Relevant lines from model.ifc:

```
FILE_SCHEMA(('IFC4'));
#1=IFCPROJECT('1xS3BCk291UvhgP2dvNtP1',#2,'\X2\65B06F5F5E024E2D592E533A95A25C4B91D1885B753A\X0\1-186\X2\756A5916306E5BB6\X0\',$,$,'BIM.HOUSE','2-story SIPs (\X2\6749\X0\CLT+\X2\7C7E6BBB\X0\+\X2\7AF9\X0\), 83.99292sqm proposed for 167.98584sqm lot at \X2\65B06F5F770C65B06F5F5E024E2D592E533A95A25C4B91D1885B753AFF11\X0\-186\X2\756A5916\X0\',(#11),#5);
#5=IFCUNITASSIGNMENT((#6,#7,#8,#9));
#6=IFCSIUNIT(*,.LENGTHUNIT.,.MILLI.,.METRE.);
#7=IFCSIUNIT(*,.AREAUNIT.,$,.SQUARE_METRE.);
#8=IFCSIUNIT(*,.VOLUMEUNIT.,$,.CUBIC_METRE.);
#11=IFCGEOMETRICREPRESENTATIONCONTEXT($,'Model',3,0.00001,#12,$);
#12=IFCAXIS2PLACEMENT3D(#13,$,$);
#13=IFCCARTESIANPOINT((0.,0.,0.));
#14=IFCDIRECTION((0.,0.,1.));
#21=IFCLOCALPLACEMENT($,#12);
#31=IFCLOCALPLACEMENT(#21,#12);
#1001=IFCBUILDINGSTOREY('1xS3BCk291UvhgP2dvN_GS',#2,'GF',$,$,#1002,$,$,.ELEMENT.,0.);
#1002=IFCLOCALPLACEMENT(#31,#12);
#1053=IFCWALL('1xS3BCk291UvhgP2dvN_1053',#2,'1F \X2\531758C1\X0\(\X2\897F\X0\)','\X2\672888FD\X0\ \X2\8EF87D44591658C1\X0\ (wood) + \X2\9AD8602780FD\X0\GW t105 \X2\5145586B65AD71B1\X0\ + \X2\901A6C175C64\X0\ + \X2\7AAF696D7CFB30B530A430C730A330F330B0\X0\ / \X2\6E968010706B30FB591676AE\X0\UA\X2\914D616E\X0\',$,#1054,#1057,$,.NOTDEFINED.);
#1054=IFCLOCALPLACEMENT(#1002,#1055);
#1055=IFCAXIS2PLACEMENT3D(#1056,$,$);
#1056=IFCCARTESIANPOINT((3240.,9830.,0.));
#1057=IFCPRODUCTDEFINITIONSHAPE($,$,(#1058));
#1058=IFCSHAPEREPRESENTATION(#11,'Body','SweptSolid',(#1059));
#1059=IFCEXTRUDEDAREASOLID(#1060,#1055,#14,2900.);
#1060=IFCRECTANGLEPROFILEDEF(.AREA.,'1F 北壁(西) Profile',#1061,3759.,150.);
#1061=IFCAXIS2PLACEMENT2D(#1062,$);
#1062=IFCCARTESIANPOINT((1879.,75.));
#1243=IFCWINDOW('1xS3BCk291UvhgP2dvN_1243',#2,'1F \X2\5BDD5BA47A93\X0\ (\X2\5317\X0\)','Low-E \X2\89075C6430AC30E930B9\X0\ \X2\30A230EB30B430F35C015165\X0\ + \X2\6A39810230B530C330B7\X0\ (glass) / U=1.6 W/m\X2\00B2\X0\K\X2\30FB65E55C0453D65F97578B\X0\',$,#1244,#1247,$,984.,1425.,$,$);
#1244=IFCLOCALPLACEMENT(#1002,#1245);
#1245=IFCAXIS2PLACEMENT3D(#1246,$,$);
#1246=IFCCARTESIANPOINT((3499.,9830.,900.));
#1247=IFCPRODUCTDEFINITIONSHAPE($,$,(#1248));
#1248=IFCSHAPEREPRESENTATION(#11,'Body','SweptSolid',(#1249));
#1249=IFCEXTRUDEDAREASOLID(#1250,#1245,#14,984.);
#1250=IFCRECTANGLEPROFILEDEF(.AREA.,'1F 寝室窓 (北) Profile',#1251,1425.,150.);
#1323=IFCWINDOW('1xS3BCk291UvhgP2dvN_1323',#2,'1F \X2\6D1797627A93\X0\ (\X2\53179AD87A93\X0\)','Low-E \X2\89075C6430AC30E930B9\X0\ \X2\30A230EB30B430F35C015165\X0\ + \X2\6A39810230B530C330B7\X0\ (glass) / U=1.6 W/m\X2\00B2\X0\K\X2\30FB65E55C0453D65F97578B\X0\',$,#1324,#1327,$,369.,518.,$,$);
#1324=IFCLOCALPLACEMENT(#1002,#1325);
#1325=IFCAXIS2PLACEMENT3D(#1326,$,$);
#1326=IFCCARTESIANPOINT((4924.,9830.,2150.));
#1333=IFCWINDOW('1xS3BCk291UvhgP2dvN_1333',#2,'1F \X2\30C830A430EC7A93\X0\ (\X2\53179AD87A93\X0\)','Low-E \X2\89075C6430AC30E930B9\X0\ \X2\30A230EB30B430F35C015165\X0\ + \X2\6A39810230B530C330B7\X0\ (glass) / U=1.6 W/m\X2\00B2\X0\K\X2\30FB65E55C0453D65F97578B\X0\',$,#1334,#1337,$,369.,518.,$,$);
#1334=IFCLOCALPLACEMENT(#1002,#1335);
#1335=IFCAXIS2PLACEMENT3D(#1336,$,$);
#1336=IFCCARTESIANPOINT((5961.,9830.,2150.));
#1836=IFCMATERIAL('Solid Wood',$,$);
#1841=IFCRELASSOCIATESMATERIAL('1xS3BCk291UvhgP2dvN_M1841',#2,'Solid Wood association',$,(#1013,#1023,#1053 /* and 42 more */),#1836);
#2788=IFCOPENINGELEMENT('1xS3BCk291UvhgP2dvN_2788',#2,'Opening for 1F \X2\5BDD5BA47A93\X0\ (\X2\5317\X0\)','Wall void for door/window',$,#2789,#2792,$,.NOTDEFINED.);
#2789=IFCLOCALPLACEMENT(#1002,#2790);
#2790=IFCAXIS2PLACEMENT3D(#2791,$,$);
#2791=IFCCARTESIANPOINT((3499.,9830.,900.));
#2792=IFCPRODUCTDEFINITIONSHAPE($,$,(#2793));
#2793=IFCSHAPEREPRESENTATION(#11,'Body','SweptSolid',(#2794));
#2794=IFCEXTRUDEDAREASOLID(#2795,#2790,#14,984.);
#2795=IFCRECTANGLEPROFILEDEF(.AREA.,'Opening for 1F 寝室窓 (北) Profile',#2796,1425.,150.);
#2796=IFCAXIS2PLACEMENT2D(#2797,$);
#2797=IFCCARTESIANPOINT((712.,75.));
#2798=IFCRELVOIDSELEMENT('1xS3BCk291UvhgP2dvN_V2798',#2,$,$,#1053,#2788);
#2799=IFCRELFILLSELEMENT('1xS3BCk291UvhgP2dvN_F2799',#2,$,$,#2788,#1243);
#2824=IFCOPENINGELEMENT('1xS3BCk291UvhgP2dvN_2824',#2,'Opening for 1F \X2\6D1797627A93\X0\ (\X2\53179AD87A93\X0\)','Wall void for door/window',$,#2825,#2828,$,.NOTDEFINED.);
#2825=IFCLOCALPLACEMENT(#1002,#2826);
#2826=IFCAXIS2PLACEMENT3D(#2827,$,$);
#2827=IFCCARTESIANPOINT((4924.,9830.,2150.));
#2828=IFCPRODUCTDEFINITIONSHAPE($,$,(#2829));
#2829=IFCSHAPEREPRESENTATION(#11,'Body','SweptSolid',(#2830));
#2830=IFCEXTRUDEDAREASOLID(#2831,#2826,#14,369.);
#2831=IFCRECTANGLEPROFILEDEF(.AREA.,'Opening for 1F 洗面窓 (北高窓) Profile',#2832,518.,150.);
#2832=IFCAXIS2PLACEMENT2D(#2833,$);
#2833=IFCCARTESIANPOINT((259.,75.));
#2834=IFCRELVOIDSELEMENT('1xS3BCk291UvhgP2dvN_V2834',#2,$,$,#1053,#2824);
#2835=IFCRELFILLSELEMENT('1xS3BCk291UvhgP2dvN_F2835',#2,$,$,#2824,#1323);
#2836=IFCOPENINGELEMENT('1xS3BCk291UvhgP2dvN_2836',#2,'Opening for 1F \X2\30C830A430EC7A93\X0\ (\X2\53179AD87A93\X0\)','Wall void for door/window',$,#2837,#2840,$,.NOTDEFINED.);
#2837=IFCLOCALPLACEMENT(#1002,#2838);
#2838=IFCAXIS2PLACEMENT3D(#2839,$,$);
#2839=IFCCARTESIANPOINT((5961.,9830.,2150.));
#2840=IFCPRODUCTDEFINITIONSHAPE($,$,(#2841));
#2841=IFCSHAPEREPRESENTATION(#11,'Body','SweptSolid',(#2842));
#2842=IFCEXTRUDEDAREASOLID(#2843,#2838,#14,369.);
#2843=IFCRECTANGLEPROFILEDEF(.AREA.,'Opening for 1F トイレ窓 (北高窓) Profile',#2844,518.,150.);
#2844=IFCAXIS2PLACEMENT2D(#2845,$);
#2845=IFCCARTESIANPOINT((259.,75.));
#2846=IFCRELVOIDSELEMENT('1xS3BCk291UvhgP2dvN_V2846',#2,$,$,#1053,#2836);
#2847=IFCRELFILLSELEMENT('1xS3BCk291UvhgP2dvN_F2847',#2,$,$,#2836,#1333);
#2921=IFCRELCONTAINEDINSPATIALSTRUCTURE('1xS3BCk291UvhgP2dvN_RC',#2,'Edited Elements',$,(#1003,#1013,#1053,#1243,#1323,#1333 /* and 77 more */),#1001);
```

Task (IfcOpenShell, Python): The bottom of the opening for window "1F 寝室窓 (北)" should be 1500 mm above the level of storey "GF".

```python
import numpy as np
import ifcopenshell
import ifcopenshell.api.geometry
import ifcopenshell.geom
import ifcopenshell.util.element
import ifcopenshell.util.placement
import ifcopenshell.util.shape
import ifcopenshell.util.unit

model = ifcopenshell.open("model.ifc")
unit_scale = ifcopenshell.util.unit.calculate_unit_scale(model)

window = model.by_guid("1xS3BCk291UvhgP2dvN_1243")
opening = window.FillsVoids[0].RelatingOpeningElement
storey = ifcopenshell.util.element.get_container(window, ifc_class="IfcBuildingStorey")
level = ifcopenshell.util.placement.get_local_placement(storey.ObjectPlacement)[2, 3]

# The opening's origin need not be at the sill, so measure its lowest point.
shape = ifcopenshell.geom.create_shape(ifcopenshell.geom.settings(), opening)
bottom = ifcopenshell.util.shape.get_shape_bottom_elevation(shape, shape.geometry) / unit_scale
dz = level + 1.5 / unit_scale - bottom

shift = np.array([0.0, 0.0, dz])
# The window is not placed relative to its opening, so move both.
for product in (opening, window):
    matrix = ifcopenshell.util.placement.get_local_placement(product.ObjectPlacement)
    matrix[:3, 3] += shift
    ifcopenshell.api.geometry.edit_object_placement(model, product=product, matrix=matrix, is_si=False)

print(f"moved by {dz * unit_scale:+.3f} m")

model.write("model_v2.ifc")
```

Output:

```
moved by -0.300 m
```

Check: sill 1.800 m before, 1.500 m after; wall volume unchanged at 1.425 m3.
